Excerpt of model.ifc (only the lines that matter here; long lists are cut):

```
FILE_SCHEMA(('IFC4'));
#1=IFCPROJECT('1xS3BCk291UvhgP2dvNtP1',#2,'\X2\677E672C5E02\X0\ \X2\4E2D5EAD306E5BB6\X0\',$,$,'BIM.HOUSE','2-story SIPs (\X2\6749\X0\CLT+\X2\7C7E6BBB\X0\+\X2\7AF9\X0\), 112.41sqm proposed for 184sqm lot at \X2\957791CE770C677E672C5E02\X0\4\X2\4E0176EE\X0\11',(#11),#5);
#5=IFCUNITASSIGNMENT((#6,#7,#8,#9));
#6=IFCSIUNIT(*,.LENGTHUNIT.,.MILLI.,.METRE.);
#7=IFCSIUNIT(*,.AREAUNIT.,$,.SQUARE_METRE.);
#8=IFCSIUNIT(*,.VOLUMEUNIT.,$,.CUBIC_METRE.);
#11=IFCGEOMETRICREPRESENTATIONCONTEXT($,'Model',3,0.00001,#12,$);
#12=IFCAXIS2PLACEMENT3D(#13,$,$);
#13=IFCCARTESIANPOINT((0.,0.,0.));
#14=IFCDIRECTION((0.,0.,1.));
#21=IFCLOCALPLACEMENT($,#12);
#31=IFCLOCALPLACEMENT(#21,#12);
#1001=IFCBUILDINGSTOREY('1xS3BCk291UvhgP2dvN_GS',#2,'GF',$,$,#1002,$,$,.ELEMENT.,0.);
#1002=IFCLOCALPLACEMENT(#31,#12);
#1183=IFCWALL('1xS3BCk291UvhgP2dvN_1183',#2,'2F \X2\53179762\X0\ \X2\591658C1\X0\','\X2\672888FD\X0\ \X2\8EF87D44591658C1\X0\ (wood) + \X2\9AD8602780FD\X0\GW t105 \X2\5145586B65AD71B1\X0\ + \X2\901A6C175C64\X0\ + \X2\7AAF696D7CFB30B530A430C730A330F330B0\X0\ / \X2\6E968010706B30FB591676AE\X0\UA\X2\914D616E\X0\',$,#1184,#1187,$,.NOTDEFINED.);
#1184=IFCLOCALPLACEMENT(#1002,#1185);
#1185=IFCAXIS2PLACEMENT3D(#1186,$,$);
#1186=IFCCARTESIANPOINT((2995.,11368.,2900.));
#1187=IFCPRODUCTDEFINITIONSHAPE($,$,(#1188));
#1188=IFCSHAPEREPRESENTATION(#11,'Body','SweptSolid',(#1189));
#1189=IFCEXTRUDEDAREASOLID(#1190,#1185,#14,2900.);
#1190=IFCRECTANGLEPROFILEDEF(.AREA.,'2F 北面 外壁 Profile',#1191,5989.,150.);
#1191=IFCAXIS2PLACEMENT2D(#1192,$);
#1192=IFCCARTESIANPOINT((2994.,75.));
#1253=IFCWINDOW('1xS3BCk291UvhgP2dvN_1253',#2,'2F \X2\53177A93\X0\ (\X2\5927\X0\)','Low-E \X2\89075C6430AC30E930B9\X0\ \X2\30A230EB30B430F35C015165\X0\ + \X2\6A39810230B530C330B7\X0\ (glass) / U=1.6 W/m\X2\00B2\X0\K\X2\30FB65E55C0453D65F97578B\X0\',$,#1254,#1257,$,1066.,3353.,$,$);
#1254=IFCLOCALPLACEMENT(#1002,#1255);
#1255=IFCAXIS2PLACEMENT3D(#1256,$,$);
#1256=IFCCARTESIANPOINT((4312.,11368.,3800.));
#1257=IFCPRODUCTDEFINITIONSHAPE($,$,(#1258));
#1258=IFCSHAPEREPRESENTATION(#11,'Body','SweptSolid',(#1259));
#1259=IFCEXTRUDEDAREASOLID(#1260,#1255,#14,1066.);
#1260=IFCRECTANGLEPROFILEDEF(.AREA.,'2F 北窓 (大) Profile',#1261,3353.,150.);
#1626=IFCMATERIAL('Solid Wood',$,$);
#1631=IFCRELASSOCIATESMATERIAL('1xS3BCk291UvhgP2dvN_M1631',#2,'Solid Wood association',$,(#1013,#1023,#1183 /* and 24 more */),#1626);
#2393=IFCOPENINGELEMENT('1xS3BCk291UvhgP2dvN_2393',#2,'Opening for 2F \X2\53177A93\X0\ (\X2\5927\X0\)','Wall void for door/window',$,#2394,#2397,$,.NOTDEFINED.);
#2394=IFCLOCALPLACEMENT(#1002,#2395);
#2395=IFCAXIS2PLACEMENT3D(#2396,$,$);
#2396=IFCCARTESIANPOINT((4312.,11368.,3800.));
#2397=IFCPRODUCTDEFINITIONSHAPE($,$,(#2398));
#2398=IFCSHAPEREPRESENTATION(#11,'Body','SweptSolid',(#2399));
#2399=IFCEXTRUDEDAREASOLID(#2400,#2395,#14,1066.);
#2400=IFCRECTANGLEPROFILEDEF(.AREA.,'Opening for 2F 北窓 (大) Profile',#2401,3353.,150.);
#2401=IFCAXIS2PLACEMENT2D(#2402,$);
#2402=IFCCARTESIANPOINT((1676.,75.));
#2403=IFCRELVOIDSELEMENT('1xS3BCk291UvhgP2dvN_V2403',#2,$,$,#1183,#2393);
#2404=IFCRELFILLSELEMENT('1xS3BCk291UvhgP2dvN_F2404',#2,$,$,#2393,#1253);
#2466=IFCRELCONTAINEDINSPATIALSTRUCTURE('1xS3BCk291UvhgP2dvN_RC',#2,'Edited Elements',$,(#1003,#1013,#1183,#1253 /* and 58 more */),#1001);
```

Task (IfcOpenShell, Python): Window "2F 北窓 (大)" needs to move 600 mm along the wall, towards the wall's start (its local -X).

```python
import ifcopenshell
import ifcopenshell.api.geometry
import ifcopenshell.util.placement

model = ifcopenshell.open("model.ifc")

window = model.by_guid("1xS3BCk291UvhgP2dvN_1253")
opening = window.FillsVoids[0].RelatingOpeningElement
wall = opening.VoidsElements[0].RelatingBuildingElement

wall_matrix = ifcopenshell.util.placement.get_local_placement(wall.ObjectPlacement)
shift = wall_matrix[:3, 0] * -600.0
before = ifcopenshell.util.placement.get_local_placement(window.ObjectPlacement)[:3, 3].copy()

# The window is not placed relative to its opening, so move both.
for product in (opening, window):
    matrix = ifcopenshell.util.placement.get_local_placement(product.ObjectPlacement)
    matrix[:3, 3] += shift
    ifcopenshell.api.geometry.edit_object_placement(model, product=product, matrix=matrix, is_si=False)

after = ifcopenshell.util.placement.get_local_placement(window.ObjectPlacement)[:3, 3]
print("window moved by", (after - before).round(3) + 0.0)

model.write("model_updated.ifc")
```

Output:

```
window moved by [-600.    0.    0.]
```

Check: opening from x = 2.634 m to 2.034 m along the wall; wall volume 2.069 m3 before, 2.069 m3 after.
